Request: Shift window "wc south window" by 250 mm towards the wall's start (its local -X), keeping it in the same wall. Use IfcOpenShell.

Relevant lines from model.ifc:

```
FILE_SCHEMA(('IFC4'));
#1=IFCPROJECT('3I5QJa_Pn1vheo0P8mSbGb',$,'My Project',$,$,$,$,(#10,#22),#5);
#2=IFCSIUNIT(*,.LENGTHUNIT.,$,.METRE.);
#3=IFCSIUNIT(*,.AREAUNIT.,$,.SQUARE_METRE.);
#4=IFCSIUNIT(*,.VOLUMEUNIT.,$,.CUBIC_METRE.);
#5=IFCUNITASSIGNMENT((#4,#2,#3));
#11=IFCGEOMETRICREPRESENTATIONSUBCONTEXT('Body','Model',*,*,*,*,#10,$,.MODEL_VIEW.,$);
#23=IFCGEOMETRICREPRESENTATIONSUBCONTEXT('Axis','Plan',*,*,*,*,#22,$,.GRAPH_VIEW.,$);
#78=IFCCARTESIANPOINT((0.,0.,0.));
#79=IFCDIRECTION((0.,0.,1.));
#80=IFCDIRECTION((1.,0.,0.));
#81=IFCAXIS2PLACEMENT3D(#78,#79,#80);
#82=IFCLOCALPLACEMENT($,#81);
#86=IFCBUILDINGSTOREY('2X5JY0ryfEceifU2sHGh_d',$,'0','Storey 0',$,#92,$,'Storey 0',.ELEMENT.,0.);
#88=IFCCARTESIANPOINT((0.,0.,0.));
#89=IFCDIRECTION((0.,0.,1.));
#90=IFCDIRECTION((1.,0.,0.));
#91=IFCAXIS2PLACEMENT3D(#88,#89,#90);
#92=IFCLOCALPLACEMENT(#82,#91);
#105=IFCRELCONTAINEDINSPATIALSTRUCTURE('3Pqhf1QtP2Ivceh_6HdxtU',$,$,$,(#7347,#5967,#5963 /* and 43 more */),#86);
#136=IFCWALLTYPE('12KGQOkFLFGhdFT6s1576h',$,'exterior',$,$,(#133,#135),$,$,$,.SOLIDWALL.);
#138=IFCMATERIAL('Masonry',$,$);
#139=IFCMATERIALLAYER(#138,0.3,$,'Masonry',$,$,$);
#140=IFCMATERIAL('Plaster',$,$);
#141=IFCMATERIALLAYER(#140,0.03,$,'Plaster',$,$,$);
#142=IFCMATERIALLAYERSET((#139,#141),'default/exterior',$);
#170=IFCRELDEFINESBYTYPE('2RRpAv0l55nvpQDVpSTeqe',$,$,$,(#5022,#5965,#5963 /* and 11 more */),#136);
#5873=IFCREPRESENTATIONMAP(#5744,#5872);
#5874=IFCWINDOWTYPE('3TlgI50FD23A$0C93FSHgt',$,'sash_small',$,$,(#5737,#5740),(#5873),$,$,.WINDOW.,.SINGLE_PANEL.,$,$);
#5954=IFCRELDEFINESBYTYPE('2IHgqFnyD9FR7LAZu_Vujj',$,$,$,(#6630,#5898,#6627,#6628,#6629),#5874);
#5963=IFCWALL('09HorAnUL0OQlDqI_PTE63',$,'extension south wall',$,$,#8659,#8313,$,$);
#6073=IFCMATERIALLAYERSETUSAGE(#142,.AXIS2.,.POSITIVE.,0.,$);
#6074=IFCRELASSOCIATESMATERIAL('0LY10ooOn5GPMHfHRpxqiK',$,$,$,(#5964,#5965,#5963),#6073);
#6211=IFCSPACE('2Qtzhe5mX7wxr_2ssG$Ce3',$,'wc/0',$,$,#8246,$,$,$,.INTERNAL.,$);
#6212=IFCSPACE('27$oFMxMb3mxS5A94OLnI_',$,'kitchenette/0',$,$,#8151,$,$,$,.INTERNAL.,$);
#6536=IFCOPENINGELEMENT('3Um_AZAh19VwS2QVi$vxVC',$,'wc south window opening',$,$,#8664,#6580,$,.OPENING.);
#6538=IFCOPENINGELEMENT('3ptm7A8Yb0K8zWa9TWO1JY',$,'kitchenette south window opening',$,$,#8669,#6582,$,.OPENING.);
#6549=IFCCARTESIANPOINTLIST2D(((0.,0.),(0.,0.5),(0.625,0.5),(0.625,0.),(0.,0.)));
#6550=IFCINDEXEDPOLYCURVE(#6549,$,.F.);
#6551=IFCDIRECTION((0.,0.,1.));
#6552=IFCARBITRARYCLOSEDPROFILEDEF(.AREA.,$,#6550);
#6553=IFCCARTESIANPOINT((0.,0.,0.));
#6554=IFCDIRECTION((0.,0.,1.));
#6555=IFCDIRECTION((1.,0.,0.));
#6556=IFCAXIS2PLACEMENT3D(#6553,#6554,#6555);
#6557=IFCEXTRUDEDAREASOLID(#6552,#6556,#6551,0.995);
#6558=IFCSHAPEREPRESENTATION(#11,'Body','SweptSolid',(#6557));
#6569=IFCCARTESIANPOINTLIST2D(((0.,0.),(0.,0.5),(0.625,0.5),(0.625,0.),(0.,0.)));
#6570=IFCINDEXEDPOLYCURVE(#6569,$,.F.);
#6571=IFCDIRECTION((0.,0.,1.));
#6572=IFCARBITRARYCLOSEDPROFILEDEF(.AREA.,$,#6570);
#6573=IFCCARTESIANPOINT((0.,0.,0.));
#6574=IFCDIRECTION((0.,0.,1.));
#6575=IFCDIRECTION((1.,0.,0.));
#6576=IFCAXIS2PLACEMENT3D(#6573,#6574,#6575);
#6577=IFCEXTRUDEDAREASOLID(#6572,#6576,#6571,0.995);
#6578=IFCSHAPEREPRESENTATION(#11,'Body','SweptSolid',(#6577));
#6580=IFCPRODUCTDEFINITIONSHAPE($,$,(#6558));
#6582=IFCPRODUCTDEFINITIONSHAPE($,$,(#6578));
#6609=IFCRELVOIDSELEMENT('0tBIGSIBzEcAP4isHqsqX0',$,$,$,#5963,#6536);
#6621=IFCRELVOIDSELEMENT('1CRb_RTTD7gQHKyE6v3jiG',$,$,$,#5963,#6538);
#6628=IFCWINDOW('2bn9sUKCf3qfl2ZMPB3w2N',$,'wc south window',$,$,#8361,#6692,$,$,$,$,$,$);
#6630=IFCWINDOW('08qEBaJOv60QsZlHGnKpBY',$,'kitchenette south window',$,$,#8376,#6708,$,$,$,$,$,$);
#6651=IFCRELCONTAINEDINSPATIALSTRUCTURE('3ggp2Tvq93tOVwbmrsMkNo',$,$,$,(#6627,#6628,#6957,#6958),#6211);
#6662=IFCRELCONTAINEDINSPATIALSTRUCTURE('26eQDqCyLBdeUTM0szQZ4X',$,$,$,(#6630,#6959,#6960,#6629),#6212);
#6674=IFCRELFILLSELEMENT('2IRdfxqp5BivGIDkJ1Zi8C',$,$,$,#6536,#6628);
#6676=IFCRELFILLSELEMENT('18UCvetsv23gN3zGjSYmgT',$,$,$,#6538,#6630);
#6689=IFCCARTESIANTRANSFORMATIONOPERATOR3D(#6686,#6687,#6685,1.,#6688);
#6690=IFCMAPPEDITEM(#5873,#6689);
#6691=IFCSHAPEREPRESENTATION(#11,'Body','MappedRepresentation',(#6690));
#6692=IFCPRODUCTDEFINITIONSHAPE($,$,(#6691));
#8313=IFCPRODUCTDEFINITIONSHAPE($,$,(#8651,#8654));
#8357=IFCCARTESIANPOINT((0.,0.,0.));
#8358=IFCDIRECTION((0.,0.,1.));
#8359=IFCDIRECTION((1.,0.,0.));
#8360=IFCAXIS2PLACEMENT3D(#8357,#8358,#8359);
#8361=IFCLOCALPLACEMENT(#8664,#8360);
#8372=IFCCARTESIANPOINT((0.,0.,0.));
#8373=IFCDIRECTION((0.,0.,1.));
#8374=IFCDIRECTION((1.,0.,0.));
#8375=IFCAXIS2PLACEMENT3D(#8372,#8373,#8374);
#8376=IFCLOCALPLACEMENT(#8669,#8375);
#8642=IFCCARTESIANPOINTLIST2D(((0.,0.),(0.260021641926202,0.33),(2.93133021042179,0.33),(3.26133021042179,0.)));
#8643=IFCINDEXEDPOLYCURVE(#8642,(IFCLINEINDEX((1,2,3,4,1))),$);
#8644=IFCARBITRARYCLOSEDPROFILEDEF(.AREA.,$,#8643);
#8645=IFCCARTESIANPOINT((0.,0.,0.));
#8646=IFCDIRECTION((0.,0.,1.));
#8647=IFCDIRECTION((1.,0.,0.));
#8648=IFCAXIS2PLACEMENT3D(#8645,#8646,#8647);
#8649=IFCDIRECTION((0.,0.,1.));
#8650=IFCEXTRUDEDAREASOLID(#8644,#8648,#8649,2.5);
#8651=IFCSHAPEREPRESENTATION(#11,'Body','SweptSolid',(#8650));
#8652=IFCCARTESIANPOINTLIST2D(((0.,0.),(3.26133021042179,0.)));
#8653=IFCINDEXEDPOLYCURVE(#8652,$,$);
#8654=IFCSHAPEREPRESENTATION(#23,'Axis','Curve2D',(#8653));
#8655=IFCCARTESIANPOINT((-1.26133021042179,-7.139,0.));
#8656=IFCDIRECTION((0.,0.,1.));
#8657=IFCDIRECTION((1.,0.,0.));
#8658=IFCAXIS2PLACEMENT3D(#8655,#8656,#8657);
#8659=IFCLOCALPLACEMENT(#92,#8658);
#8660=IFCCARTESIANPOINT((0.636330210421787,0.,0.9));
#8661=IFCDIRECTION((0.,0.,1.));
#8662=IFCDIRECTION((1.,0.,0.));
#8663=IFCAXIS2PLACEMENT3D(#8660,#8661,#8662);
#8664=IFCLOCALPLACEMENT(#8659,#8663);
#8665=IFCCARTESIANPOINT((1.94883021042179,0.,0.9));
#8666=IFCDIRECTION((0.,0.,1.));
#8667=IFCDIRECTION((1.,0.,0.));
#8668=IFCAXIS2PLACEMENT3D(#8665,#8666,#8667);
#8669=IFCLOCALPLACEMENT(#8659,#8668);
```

```python
import ifcopenshell
import ifcopenshell.api.geometry
import ifcopenshell.util.placement
import ifcopenshell.util.unit

model = ifcopenshell.open("model.ifc")
unit_scale = ifcopenshell.util.unit.calculate_unit_scale(model)

window = model.by_guid("2bn9sUKCf3qfl2ZMPB3w2N")
opening = window.FillsVoids[0].RelatingOpeningElement
wall = opening.VoidsElements[0].RelatingBuildingElement

wall_matrix = ifcopenshell.util.placement.get_local_placement(wall.ObjectPlacement)
shift = wall_matrix[:3, 0] * -0.25 / unit_scale
before = ifcopenshell.util.placement.get_local_placement(window.ObjectPlacement)[:3, 3].copy()

# The window is placed relative to its opening, so it follows when the opening moves.
matrix = ifcopenshell.util.placement.get_local_placement(opening.ObjectPlacement)
matrix[:3, 3] += shift
ifcopenshell.api.geometry.edit_object_placement(
    model, product=opening, matrix=matrix, is_si=False, should_transform_children=True
)

after = ifcopenshell.util.placement.get_local_placement(window.ObjectPlacement)[:3, 3]
print("window moved by", (after - before).round(3) + 0.0)

model.write("model_updated.ifc")
```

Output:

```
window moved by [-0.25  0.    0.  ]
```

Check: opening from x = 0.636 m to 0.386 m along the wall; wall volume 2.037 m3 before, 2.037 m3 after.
